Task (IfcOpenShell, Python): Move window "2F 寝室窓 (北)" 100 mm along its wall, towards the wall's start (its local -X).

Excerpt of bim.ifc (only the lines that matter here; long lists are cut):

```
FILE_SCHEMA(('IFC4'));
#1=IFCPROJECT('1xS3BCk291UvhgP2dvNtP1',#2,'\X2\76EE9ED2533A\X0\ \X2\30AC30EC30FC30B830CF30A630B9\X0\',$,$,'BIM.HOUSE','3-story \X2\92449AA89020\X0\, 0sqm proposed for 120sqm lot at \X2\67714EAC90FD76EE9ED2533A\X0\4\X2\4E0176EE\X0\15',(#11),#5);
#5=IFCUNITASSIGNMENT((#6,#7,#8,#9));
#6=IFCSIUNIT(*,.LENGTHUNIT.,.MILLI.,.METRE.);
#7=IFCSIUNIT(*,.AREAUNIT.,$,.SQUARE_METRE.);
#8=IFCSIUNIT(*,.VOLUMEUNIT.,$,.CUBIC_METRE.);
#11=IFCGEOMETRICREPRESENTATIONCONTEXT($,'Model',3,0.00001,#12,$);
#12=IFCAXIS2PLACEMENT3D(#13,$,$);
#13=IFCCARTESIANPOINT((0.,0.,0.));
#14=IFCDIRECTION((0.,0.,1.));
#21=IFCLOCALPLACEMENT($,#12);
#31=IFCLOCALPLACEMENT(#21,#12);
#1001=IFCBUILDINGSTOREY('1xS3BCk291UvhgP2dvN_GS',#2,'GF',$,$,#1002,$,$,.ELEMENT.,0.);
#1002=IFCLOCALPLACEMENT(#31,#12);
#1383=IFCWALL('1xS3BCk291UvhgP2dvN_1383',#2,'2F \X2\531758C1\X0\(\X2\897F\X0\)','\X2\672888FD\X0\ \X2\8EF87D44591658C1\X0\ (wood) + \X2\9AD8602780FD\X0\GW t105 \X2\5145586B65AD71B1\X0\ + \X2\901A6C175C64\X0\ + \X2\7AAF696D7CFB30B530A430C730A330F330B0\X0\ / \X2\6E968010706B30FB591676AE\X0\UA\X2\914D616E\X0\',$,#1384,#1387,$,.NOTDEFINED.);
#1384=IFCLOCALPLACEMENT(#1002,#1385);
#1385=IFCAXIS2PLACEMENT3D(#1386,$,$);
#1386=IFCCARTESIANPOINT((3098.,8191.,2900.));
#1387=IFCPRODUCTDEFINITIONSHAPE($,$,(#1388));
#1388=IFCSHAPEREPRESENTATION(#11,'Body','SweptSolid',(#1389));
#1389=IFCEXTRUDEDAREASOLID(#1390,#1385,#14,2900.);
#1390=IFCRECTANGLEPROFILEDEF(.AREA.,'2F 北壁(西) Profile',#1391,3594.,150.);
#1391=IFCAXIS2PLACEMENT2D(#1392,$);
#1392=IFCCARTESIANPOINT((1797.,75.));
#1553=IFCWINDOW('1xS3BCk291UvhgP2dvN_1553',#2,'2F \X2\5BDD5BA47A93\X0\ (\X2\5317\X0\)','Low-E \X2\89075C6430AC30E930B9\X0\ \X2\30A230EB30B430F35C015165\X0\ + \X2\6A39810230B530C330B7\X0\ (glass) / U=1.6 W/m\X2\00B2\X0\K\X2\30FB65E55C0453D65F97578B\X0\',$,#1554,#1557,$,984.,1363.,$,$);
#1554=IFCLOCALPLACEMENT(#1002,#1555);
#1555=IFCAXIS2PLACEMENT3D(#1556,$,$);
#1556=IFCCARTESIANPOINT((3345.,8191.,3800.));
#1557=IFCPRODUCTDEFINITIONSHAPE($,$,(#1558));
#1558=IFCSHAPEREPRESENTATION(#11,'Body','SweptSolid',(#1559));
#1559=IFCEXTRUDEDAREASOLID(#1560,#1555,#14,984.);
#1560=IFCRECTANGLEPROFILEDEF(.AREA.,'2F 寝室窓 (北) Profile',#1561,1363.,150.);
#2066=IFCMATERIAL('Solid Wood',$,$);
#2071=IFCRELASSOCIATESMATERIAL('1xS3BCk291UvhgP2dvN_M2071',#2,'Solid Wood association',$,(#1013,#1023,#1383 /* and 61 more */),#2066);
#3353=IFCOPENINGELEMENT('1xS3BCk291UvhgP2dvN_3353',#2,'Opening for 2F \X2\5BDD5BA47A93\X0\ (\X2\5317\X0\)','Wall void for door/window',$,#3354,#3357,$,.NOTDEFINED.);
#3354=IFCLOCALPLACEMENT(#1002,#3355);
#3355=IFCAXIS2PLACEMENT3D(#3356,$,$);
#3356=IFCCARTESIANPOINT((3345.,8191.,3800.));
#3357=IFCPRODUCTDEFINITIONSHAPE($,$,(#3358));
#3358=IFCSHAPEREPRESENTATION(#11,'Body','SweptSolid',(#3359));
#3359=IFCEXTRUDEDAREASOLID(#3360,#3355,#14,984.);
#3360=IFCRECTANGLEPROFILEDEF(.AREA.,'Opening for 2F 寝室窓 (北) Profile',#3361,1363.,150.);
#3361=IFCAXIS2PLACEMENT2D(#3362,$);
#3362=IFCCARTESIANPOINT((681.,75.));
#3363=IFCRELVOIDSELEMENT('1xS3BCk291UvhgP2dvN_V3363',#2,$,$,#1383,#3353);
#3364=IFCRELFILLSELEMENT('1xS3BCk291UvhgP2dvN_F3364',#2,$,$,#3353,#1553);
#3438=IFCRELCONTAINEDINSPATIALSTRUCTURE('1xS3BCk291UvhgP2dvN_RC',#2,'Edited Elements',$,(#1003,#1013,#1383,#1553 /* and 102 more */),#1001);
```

```python
import ifcopenshell
import ifcopenshell.api.geometry
import ifcopenshell.util.placement

model = ifcopenshell.open("bim.ifc")

window = model.by_guid("1xS3BCk291UvhgP2dvN_1553")
opening = window.FillsVoids[0].RelatingOpeningElement
wall = opening.VoidsElements[0].RelatingBuildingElement

wall_matrix = ifcopenshell.util.placement.get_local_placement(wall.ObjectPlacement)
shift = wall_matrix[:3, 0] * -100.0
before = ifcopenshell.util.placement.get_local_placement(window.ObjectPlacement)[:3, 3].copy()

# The window is not placed relative to its opening, so move both.
for product in (opening, window):
    matrix = ifcopenshell.util.placement.get_local_placement(product.ObjectPlacement)
    matrix[:3, 3] += shift
    ifcopenshell.api.geometry.edit_object_placement(model, product=product, matrix=matrix, is_si=False)

after = ifcopenshell.util.placement.get_local_placement(window.ObjectPlacement)[:3, 3]
print("window moved by", (after - before).round(3) + 0.0)

model.write("bim_v2.ifc")
```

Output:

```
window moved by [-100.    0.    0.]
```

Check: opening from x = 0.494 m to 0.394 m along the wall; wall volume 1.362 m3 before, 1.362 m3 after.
